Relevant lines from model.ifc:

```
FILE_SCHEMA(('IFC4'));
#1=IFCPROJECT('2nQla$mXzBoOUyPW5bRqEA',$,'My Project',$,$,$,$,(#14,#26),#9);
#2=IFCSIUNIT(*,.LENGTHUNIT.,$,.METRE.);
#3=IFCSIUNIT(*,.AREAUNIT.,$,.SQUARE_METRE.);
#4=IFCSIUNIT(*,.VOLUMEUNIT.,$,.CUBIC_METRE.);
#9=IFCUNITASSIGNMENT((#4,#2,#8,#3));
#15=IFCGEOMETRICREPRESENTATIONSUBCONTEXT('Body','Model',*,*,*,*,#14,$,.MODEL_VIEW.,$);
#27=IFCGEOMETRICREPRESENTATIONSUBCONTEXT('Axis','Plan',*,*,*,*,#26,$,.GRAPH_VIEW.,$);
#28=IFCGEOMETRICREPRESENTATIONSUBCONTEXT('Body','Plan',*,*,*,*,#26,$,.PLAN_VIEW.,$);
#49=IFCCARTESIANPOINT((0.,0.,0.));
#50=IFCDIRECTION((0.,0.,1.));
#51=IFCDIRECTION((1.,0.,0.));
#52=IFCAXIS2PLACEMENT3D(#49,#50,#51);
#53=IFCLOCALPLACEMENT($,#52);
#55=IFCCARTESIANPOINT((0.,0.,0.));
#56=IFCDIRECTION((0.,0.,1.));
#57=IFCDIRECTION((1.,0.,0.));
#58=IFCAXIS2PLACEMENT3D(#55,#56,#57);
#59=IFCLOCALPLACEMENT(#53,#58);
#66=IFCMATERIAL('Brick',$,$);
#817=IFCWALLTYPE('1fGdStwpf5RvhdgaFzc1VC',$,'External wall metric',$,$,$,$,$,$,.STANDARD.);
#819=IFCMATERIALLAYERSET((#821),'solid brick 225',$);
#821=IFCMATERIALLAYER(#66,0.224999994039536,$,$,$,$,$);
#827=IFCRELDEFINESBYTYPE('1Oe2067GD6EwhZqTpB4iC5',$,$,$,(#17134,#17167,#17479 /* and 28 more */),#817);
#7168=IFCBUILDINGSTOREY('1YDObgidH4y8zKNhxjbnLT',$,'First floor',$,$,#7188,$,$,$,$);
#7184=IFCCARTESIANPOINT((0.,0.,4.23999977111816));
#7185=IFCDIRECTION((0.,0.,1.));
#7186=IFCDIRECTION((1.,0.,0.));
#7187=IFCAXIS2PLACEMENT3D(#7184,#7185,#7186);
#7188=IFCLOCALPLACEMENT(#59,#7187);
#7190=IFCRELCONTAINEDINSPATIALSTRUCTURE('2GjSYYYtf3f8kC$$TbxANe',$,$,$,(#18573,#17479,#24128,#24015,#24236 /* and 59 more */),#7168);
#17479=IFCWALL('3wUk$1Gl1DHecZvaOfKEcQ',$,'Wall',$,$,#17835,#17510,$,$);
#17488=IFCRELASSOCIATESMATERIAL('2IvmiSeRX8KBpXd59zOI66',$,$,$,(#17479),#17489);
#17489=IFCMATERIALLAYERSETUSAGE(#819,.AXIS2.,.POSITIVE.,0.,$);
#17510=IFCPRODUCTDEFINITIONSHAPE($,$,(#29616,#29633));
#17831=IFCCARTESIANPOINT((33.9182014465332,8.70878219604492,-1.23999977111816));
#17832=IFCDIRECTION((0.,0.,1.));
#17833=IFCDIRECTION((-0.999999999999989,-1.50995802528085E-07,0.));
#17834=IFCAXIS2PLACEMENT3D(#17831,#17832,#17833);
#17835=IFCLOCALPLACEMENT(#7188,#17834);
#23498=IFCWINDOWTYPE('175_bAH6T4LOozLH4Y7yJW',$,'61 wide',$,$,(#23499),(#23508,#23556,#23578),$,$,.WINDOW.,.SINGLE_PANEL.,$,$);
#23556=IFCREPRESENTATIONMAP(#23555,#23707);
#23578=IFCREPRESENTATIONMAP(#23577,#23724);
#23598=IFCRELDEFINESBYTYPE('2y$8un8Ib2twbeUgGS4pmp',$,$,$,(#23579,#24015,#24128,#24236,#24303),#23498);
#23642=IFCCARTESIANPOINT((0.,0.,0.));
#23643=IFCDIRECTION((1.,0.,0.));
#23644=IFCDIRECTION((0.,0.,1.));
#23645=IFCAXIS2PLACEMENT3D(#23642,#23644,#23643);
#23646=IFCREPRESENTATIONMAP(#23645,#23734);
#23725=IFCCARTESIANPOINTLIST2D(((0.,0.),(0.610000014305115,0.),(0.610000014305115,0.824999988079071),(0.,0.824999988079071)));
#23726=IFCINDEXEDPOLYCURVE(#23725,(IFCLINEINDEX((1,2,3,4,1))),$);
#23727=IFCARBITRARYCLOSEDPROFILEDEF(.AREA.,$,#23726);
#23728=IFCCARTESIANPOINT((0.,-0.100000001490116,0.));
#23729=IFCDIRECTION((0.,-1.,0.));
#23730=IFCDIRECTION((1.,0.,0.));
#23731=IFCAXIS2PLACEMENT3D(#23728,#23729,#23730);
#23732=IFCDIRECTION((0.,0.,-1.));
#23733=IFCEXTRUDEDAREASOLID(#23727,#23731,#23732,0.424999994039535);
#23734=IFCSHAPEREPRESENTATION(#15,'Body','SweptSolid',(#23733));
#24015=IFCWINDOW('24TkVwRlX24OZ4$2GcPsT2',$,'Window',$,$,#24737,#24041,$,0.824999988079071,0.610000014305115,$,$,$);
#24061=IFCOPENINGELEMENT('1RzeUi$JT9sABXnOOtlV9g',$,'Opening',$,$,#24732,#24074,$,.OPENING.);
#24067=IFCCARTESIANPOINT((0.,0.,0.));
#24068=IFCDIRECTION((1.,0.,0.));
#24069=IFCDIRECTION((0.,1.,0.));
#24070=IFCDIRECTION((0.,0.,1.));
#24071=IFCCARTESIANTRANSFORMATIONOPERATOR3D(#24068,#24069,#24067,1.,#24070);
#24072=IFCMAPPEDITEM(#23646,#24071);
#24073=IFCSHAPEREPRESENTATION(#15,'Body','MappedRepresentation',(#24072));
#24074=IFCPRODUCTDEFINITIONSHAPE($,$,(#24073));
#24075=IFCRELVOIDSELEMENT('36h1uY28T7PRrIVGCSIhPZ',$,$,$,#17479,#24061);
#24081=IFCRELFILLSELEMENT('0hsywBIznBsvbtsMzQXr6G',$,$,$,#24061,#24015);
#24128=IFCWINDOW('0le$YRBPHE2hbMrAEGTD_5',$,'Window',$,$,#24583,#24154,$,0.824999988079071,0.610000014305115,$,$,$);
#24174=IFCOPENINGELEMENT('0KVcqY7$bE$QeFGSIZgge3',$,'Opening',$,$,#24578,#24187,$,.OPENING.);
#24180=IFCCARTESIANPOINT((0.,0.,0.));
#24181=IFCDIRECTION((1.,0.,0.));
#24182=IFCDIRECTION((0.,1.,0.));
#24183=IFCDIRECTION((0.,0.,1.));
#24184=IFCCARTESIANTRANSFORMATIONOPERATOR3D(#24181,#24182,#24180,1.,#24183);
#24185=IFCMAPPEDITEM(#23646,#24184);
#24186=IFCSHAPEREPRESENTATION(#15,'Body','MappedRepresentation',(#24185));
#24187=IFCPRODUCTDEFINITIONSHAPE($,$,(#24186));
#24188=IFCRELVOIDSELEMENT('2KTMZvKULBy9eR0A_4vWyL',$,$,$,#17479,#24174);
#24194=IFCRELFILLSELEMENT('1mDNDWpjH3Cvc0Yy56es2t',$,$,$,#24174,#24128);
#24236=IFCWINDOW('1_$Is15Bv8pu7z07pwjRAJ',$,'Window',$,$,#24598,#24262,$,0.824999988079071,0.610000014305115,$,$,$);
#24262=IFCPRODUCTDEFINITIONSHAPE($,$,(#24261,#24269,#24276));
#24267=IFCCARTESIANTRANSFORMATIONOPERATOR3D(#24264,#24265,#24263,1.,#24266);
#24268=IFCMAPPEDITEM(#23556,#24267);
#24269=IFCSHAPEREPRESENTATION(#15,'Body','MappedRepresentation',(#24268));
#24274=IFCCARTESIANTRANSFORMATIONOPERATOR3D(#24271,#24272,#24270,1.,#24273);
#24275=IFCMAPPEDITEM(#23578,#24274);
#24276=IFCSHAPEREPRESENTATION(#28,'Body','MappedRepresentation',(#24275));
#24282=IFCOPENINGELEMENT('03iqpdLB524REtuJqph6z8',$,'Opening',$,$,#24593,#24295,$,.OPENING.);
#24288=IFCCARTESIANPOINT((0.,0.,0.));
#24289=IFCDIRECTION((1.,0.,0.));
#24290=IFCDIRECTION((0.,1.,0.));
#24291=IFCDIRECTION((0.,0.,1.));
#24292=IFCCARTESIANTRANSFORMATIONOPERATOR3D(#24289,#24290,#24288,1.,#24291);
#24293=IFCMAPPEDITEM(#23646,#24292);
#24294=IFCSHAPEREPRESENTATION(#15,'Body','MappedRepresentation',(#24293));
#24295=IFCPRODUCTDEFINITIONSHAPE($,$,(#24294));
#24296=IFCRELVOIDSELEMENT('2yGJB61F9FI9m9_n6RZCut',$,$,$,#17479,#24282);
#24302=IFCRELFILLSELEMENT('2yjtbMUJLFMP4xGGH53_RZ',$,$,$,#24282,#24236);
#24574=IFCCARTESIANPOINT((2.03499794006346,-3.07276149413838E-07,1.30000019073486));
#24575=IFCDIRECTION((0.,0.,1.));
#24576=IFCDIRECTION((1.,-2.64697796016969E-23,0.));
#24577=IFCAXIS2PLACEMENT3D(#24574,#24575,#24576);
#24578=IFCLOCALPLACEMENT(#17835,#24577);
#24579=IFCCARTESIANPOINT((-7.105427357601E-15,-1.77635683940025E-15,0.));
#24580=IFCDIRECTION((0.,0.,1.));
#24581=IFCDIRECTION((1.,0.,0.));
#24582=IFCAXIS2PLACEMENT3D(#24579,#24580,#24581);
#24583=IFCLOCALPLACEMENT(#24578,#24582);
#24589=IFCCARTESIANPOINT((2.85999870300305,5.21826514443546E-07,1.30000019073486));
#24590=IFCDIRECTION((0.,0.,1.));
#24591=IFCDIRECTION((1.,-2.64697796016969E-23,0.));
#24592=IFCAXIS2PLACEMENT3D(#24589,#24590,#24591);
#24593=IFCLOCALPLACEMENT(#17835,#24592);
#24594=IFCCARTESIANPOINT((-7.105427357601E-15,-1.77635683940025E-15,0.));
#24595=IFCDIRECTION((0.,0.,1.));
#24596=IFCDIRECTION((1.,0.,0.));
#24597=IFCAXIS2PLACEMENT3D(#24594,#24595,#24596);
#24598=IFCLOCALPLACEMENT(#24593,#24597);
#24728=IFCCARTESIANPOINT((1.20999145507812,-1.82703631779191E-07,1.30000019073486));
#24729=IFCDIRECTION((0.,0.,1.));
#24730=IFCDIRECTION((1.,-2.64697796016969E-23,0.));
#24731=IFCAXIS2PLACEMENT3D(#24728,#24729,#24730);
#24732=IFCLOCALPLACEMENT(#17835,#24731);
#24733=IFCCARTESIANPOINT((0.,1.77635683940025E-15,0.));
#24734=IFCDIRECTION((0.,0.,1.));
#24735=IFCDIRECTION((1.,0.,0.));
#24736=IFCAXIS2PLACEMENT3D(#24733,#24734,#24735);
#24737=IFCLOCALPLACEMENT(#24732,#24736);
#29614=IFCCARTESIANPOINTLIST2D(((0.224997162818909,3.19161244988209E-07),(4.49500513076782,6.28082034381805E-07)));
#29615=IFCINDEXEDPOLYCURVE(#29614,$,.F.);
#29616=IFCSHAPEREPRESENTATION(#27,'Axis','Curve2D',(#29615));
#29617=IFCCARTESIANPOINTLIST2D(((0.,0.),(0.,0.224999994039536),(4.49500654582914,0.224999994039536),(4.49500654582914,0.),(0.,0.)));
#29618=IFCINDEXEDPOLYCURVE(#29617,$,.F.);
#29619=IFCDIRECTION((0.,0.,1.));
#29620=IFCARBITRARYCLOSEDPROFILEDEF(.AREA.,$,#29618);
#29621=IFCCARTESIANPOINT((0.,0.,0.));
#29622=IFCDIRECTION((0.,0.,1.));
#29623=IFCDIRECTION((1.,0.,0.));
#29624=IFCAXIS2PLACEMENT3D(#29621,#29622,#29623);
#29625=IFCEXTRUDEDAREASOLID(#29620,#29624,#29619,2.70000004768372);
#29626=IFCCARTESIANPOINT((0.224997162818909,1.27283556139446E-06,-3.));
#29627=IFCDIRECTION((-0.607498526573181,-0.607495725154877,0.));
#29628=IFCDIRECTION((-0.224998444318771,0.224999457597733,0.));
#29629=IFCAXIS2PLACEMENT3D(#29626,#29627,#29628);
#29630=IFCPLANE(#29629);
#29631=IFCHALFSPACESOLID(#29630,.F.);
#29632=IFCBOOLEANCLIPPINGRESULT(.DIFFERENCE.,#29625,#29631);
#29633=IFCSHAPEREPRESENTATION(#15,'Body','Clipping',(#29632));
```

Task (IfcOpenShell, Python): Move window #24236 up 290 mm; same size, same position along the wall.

```python
import numpy as np
import ifcopenshell
import ifcopenshell.api.geometry
import ifcopenshell.util.placement
import ifcopenshell.util.unit

model = ifcopenshell.open("model.ifc")
unit_scale = ifcopenshell.util.unit.calculate_unit_scale(model)

window = model.by_guid("1_$Is15Bv8pu7z07pwjRAJ")
opening = window.FillsVoids[0].RelatingOpeningElement
dz = 0.29 / unit_scale

shift = np.array([0.0, 0.0, dz])
# The window is placed relative to its opening, so it follows when the opening moves.
matrix = ifcopenshell.util.placement.get_local_placement(opening.ObjectPlacement)
matrix[:3, 3] += shift
ifcopenshell.api.geometry.edit_object_placement(
    model, product=opening, matrix=matrix, is_si=False, should_transform_children=True
)

print(f"moved by {dz * unit_scale:+.3f} m")

model.write("model_edited.ifc")
```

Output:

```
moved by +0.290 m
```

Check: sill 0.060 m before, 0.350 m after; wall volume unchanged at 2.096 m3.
